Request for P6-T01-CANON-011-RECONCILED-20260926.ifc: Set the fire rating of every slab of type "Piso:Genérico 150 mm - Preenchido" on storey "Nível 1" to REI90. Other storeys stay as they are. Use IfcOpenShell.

First a look at what the model holds.

```python
import ifcopenshell
import ifcopenshell.util.element

model = ifcopenshell.open("P6-T01-CANON-011-RECONCILED-20260926.ifc")
print(model.schema)
storey = next(s for s in model.by_type("IfcBuildingStorey") if s.Name == "Nível 1")
slabs = [e for e in ifcopenshell.util.element.get_decomposition(storey) if e.is_a("IfcSlab")]
seen = {}
for e in slabs:
    element_type = ifcopenshell.util.element.get_type(e)
    key = (element_type.Name if element_type != e and element_type else None, ifcopenshell.util.element.get_pset(e, "Pset_SlabCommon", "FireRating"))
    seen[key] = seen.get(key, 0) + 1
for (name, value), count in sorted(seen.items(), key=str):
    print(count, "x", name, "|", value)
```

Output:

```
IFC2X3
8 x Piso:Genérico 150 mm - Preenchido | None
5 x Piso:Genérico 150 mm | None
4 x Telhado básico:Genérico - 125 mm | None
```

```python
import ifcopenshell
import ifcopenshell.api.pset
import ifcopenshell.util.element

model = ifcopenshell.open("P6-T01-CANON-011-RECONCILED-20260926.ifc")

storey = next(s for s in model.by_type("IfcBuildingStorey") if s.Name == "Nível 1")
slabs = [e for e in ifcopenshell.util.element.get_decomposition(storey) if e.is_a("IfcSlab")]

count = 0
for e in slabs:
    element_type = ifcopenshell.util.element.get_type(e)
    if element_type in (None, e) or element_type.Name != "Piso:Genérico 150 mm - Preenchido":
        continue
    # add_pset returns the element's existing set when there is one.
    pset = ifcopenshell.api.pset.add_pset(model, product=e, name="Pset_SlabCommon")
    ifcopenshell.api.pset.edit_pset(model, pset=pset, properties={"FireRating": "REI90"})
    count += 1

print(count, "slabs updated")

model.write("P6-T01-CANON-011-RECONCILED-20260926_updated.ifc")
```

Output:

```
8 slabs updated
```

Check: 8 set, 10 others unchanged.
